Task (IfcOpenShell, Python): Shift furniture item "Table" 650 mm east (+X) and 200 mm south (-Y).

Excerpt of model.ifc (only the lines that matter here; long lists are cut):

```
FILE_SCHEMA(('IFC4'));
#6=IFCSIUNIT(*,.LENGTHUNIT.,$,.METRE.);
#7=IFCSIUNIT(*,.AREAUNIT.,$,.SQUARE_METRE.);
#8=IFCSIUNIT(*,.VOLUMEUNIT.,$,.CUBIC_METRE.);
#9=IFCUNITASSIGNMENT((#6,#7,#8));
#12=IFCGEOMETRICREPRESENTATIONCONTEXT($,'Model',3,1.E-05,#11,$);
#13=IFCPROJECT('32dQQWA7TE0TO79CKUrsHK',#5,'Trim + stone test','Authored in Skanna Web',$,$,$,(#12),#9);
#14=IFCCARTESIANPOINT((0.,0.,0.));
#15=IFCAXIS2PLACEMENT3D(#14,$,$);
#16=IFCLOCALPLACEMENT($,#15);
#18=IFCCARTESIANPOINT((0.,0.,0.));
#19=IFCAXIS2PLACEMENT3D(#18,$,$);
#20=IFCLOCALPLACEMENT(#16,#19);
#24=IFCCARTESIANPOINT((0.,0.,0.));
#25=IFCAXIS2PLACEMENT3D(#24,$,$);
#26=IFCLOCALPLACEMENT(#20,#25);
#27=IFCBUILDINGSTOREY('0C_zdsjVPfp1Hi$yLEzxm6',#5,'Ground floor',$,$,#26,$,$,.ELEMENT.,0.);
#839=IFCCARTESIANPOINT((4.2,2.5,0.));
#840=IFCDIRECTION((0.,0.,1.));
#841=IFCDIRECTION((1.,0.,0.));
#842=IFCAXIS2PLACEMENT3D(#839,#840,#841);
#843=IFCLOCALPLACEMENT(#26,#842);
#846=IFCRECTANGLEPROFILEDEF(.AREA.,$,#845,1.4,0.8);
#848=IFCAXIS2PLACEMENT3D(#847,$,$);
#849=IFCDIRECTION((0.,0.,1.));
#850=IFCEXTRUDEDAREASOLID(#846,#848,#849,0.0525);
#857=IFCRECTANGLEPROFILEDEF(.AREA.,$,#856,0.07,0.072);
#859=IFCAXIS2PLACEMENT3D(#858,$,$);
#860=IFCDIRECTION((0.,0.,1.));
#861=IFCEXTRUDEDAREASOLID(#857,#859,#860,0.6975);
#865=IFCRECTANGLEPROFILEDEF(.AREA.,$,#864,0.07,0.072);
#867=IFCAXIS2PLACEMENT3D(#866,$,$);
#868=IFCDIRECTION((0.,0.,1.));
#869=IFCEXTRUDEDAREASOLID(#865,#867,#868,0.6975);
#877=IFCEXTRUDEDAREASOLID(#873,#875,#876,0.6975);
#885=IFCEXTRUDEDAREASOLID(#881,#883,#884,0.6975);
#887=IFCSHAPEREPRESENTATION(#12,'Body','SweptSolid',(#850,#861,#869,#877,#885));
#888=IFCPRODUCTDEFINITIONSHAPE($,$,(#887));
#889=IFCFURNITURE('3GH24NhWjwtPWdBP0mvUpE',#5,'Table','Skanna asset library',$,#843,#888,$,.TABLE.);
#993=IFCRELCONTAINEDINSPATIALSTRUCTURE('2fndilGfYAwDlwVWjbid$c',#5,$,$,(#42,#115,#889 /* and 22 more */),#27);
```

```python
import ifcopenshell
import ifcopenshell.api.geometry
import ifcopenshell.util.placement
import ifcopenshell.util.unit

model = ifcopenshell.open("model.ifc")
unit_scale = ifcopenshell.util.unit.calculate_unit_scale(model)

item = model.by_guid("3GH24NhWjwtPWdBP0mvUpE")
matrix = ifcopenshell.util.placement.get_local_placement(item.ObjectPlacement)
matrix[0, 3] += 0.65 / unit_scale
matrix[1, 3] -= 0.2 / unit_scale
ifcopenshell.api.geometry.edit_object_placement(model, product=item, matrix=matrix, is_si=False)

print(ifcopenshell.util.placement.get_local_placement(item.ObjectPlacement).round(3) + 0.0)

model.write("model_edited.ifc")
```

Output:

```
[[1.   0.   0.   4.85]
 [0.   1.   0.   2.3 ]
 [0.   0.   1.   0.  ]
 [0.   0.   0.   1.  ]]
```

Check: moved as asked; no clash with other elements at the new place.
